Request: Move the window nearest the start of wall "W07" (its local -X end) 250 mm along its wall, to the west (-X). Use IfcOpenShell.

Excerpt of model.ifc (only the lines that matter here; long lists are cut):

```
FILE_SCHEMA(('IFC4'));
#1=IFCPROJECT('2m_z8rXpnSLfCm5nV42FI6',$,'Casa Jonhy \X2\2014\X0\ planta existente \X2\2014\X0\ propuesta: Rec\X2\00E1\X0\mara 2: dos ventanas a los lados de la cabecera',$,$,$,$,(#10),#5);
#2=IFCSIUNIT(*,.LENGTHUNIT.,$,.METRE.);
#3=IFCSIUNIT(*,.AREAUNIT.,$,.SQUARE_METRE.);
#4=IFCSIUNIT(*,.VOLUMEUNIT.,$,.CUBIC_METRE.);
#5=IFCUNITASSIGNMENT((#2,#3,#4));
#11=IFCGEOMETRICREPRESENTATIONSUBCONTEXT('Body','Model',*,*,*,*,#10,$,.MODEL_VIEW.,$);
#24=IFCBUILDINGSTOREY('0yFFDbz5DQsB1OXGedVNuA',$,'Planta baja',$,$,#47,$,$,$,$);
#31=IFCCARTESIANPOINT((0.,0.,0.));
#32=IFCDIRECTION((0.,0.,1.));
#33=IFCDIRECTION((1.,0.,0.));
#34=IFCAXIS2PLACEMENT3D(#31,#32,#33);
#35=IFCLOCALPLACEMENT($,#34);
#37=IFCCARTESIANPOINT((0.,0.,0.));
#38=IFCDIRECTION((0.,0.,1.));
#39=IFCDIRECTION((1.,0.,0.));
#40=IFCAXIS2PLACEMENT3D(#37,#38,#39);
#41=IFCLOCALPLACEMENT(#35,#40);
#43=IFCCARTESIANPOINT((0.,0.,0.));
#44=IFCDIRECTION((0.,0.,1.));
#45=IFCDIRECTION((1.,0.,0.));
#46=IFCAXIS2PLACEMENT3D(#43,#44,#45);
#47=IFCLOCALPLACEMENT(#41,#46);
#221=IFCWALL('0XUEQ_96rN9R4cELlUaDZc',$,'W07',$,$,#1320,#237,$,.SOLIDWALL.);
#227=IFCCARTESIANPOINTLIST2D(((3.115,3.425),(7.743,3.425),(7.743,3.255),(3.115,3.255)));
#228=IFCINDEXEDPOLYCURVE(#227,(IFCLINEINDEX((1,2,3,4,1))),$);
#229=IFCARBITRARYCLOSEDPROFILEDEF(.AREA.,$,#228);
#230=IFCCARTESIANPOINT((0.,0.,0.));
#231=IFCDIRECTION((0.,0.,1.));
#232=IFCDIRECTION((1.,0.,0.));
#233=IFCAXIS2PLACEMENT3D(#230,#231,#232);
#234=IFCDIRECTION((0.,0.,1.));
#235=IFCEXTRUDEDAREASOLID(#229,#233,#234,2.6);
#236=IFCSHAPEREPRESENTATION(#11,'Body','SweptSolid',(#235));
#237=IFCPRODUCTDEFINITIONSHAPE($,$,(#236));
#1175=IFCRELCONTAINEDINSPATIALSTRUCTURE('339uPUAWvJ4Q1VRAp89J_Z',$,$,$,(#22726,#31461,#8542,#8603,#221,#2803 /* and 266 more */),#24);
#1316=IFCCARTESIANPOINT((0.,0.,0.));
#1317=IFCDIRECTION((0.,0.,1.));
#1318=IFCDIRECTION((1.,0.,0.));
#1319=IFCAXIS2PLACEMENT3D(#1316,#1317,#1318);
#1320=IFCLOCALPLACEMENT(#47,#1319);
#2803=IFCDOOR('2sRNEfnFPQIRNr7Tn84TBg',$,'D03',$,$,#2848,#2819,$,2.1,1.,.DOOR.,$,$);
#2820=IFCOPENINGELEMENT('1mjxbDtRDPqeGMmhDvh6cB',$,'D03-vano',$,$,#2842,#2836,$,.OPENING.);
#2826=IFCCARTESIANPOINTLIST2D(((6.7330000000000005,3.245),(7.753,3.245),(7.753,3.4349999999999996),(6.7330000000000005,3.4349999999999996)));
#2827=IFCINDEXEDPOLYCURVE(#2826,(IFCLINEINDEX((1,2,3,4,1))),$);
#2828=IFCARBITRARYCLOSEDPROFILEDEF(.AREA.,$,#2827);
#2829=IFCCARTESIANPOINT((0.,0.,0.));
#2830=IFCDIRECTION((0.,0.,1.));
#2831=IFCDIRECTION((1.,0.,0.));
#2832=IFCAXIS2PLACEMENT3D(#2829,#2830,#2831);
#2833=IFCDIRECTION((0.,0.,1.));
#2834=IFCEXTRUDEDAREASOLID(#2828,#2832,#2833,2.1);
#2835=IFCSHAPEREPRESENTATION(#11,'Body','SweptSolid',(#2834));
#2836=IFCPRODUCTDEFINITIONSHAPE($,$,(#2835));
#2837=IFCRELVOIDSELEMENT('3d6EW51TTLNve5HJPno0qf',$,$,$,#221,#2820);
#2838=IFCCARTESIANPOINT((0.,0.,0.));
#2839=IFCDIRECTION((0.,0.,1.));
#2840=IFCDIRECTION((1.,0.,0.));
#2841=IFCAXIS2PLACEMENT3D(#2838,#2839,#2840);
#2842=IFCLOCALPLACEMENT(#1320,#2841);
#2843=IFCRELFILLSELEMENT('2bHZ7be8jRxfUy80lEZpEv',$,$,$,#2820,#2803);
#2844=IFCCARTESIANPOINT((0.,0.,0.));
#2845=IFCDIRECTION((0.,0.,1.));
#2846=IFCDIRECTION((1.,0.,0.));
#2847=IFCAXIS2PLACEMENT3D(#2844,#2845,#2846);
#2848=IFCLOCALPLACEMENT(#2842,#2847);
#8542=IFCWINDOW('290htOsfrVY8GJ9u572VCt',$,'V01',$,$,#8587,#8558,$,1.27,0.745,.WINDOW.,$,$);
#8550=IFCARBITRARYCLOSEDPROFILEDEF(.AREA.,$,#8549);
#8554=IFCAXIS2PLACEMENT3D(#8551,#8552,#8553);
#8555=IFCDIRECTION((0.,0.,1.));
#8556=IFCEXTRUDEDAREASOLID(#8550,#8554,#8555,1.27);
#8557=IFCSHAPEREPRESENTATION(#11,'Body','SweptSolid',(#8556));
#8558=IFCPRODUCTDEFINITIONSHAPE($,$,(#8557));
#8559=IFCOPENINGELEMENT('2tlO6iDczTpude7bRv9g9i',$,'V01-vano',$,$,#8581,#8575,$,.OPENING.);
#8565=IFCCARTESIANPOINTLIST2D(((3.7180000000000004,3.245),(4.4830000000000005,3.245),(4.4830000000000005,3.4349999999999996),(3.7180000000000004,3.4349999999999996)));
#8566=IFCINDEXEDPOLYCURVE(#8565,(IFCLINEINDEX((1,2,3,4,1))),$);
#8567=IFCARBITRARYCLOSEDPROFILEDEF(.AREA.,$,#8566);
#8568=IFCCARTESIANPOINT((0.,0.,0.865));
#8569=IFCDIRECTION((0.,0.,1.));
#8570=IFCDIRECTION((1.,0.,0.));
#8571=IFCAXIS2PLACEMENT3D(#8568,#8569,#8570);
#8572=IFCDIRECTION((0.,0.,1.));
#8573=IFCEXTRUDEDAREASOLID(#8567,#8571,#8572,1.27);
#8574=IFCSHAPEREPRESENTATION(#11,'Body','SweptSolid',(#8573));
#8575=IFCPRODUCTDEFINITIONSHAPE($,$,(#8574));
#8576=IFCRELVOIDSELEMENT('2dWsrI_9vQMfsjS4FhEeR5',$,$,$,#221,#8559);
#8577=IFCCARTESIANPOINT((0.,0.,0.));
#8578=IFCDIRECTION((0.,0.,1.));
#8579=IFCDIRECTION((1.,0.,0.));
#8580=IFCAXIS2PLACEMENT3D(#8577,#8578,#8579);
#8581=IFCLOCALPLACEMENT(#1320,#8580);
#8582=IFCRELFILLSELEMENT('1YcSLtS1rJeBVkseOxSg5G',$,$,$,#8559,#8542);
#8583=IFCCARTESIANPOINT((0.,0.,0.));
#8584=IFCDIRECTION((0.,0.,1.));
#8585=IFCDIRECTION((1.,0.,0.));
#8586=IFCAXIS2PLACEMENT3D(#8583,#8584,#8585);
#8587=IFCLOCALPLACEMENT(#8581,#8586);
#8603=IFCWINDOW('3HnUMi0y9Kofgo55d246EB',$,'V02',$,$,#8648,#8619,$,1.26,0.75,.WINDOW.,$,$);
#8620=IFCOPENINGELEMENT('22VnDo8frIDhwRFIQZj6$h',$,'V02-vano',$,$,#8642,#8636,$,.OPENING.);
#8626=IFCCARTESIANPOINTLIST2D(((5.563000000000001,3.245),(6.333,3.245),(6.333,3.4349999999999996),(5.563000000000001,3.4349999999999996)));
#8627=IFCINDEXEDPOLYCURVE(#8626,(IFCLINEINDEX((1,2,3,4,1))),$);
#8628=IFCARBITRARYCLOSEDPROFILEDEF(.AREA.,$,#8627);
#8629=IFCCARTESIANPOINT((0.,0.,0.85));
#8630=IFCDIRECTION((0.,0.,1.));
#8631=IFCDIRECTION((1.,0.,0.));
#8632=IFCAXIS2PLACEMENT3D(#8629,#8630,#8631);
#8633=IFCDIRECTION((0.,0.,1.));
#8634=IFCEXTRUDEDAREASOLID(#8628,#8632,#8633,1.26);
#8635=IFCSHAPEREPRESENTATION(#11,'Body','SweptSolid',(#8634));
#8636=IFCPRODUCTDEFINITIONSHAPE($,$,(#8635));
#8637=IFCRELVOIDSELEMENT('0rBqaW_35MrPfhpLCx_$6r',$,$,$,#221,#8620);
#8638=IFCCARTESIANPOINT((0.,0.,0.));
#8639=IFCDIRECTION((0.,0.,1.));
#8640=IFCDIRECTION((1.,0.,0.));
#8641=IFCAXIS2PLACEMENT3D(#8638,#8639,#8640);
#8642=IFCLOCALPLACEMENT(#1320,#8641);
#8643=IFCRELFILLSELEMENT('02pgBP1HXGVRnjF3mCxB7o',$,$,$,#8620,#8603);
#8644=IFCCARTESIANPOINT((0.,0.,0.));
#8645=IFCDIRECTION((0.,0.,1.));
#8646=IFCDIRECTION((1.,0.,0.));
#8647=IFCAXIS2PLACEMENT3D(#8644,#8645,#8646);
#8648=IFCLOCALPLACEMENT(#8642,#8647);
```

```python
import ifcopenshell
import ifcopenshell.api.geometry
import ifcopenshell.util.placement

model = ifcopenshell.open("model.ifc")

window = model.by_guid("290htOsfrVY8GJ9u572VCt")
opening = window.FillsVoids[0].RelatingOpeningElement
wall = opening.VoidsElements[0].RelatingBuildingElement

wall_matrix = ifcopenshell.util.placement.get_local_placement(wall.ObjectPlacement)
shift = wall_matrix[:3, 0] * -0.25
before = ifcopenshell.util.placement.get_local_placement(window.ObjectPlacement)[:3, 3].copy()

# The window is placed relative to its opening, so it follows when the opening moves.
matrix = ifcopenshell.util.placement.get_local_placement(opening.ObjectPlacement)
matrix[:3, 3] += shift
ifcopenshell.api.geometry.edit_object_placement(
    model, product=opening, matrix=matrix, is_si=False, should_transform_children=True
)

after = ifcopenshell.util.placement.get_local_placement(window.ObjectPlacement)[:3, 3]
print("window moved by", (after - before).round(3) + 0.0)

model.write("model-out.ifc")
```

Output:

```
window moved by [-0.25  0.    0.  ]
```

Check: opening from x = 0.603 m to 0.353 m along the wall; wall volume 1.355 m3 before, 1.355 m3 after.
